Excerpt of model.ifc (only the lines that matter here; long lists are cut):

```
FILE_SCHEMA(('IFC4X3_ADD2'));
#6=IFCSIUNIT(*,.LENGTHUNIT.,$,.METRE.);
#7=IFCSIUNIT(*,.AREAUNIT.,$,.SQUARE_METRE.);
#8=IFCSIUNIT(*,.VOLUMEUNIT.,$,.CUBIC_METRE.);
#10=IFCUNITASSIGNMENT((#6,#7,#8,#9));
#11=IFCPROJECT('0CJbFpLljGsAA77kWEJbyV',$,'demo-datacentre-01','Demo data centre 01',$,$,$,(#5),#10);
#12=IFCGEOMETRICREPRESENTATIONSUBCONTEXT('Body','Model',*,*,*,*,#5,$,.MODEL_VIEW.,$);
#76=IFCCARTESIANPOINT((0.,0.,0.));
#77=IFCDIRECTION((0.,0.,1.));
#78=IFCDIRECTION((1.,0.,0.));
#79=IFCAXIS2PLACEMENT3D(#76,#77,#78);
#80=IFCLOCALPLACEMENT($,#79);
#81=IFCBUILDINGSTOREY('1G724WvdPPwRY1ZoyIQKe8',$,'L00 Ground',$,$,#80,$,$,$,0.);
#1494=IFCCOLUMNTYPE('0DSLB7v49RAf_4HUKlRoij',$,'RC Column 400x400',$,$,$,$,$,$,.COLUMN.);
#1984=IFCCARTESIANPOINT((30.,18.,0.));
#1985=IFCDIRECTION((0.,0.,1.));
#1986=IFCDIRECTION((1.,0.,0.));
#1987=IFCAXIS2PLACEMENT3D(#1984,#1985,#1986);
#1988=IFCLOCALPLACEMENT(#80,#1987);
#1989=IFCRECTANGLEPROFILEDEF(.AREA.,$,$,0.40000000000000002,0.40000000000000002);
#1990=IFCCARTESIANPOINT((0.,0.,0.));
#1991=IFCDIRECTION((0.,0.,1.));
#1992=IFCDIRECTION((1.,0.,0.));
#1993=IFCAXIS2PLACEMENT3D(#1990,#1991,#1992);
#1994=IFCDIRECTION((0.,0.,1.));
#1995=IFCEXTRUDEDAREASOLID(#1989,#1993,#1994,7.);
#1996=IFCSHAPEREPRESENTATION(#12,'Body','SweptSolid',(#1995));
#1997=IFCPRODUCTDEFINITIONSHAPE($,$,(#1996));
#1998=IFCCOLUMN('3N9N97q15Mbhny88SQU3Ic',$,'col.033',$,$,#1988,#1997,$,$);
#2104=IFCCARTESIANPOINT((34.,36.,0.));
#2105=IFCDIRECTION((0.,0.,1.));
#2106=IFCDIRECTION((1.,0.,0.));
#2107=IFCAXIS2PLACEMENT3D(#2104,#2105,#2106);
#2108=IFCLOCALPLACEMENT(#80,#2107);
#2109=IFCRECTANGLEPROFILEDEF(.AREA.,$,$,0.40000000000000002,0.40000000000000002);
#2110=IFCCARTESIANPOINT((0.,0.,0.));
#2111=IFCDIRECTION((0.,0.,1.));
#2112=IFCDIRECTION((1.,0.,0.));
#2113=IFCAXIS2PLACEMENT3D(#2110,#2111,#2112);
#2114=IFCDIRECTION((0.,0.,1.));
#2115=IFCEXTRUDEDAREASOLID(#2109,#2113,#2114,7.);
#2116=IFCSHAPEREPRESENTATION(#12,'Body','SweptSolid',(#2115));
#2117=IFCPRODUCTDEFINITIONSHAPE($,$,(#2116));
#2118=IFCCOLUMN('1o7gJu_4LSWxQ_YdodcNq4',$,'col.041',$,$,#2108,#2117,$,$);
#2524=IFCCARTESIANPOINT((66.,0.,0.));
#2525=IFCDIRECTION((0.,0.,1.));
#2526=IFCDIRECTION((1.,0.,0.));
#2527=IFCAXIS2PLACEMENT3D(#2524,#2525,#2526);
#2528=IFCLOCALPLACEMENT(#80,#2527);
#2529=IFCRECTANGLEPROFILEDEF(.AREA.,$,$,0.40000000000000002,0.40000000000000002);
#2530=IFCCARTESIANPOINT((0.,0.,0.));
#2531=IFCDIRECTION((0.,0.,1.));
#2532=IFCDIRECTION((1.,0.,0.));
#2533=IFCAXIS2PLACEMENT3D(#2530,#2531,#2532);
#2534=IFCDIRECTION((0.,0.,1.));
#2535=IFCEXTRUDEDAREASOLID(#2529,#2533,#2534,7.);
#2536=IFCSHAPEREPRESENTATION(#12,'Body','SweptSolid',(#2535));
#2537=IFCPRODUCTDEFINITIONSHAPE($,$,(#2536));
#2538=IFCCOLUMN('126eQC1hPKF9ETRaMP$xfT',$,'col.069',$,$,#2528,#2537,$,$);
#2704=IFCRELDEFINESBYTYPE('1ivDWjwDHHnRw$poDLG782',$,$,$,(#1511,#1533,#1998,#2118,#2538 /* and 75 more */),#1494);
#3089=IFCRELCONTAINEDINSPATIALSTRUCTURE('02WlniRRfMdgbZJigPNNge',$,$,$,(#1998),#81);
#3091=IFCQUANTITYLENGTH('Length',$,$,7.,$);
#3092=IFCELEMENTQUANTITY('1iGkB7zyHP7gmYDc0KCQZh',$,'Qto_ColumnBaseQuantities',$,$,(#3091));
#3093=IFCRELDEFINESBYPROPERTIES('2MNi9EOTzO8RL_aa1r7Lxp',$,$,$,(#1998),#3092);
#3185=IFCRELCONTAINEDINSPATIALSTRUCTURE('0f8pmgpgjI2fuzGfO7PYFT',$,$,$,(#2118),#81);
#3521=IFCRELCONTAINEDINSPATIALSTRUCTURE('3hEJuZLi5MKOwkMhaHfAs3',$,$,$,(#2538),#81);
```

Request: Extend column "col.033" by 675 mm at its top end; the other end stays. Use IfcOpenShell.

```python
import ifcopenshell
import ifcopenshell.api.pset
import ifcopenshell.util.element
import ifcopenshell.util.representation

model = ifcopenshell.open("model.ifc")

member = model.by_guid("3N9N97q15Mbhny88SQU3Ic")
change = 0.675

# The extrusion runs towards the end named, so only its depth changes.
body = ifcopenshell.util.representation.get_representation(member, "Model", "Body")
solid = body.Items[0]
old_length = solid.Depth
solid.Depth += change

# Update the stored length and volume.
qto = model.by_id(ifcopenshell.util.element.get_pset(member, "Qto_ColumnBaseQuantities", should_inherit=False)["id"])
ifcopenshell.api.pset.edit_qto(model, qto=qto, properties={"Length": solid.Depth})

print(f"length {old_length:g} -> {solid.Depth:g}")

model.write("model_v2.ifc")
```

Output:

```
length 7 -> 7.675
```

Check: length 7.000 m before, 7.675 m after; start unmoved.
